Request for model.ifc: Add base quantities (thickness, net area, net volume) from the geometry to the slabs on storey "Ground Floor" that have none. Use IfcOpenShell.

First a look at what the model holds.

```python
import ifcopenshell
import ifcopenshell.util.element
import ifcopenshell.util.unit

model = ifcopenshell.open("model.ifc")
print(model.schema)
for unit_type in ("LENGTHUNIT", "AREAUNIT", "VOLUMEUNIT"):
    print(unit_type, ifcopenshell.util.unit.calculate_unit_scale(model, unit_type))
storey = next(s for s in model.by_type("IfcBuildingStorey") if s.Name == "Ground Floor")
slabs = [e for e in ifcopenshell.util.element.get_decomposition(storey) if e.is_a("IfcSlab")]
for e in sorted(slabs, key=lambda e: e.id()):
    print(e.id(), e.is_a(), e.Name, list(ifcopenshell.util.element.get_psets(e, qtos_only=True)), sep=" | ")
```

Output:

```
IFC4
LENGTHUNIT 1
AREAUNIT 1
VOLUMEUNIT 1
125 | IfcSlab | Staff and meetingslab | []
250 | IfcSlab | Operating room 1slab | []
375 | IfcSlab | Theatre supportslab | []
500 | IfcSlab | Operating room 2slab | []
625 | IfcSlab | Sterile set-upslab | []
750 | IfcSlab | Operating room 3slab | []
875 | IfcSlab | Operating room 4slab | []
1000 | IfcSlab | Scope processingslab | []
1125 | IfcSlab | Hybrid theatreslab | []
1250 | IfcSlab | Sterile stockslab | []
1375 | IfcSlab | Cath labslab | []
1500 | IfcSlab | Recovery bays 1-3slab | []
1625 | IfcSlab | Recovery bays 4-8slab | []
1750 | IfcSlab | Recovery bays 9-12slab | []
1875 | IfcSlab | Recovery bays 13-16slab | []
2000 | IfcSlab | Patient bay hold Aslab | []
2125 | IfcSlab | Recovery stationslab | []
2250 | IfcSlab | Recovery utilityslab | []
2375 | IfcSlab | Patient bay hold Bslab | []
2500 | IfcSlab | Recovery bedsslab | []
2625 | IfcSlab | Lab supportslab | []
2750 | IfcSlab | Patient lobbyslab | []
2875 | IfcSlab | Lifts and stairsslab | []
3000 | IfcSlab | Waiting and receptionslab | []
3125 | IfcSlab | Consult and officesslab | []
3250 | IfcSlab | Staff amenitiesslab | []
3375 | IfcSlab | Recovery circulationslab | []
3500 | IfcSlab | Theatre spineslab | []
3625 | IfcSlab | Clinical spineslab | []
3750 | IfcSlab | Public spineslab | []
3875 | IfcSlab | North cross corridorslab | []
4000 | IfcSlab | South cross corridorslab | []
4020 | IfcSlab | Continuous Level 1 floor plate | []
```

```python
import ifcopenshell
import ifcopenshell.api.pset
import ifcopenshell.geom
import ifcopenshell.util.element
import ifcopenshell.util.shape
import ifcopenshell.util.unit

model = ifcopenshell.open("model.ifc")
unit_scale = ifcopenshell.util.unit.calculate_unit_scale(model)
area_scale = ifcopenshell.util.unit.calculate_unit_scale(model, "AREAUNIT")
volume_scale = ifcopenshell.util.unit.calculate_unit_scale(model, "VOLUMEUNIT")
settings = ifcopenshell.geom.settings()

storey = next(s for s in model.by_type("IfcBuildingStorey") if s.Name == "Ground Floor")
slabs = [e for e in ifcopenshell.util.element.get_decomposition(storey) if e.is_a("IfcSlab")]

for e in sorted(slabs, key=lambda e: e.id()):
    if ifcopenshell.util.element.get_psets(e, qtos_only=True, should_inherit=False):
        continue
    # Geometry comes back in metres, in the element's own axes.
    shape = ifcopenshell.geom.create_shape(settings, e)
    values = {
        "Width": ifcopenshell.util.shape.get_z(shape.geometry) / unit_scale,
        "NetArea": ifcopenshell.util.shape.get_footprint_area(shape.geometry) / area_scale,
        "NetVolume": ifcopenshell.util.shape.get_volume(shape.geometry) / volume_scale,
    }
    qto = ifcopenshell.api.pset.add_qto(model, product=e, name="Qto_SlabBaseQuantities")
    ifcopenshell.api.pset.edit_qto(model, qto=qto, properties=values)
    print(e.id(), {k: round(v, 3) for k, v in values.items()})

model.write("model-out.ifc")
```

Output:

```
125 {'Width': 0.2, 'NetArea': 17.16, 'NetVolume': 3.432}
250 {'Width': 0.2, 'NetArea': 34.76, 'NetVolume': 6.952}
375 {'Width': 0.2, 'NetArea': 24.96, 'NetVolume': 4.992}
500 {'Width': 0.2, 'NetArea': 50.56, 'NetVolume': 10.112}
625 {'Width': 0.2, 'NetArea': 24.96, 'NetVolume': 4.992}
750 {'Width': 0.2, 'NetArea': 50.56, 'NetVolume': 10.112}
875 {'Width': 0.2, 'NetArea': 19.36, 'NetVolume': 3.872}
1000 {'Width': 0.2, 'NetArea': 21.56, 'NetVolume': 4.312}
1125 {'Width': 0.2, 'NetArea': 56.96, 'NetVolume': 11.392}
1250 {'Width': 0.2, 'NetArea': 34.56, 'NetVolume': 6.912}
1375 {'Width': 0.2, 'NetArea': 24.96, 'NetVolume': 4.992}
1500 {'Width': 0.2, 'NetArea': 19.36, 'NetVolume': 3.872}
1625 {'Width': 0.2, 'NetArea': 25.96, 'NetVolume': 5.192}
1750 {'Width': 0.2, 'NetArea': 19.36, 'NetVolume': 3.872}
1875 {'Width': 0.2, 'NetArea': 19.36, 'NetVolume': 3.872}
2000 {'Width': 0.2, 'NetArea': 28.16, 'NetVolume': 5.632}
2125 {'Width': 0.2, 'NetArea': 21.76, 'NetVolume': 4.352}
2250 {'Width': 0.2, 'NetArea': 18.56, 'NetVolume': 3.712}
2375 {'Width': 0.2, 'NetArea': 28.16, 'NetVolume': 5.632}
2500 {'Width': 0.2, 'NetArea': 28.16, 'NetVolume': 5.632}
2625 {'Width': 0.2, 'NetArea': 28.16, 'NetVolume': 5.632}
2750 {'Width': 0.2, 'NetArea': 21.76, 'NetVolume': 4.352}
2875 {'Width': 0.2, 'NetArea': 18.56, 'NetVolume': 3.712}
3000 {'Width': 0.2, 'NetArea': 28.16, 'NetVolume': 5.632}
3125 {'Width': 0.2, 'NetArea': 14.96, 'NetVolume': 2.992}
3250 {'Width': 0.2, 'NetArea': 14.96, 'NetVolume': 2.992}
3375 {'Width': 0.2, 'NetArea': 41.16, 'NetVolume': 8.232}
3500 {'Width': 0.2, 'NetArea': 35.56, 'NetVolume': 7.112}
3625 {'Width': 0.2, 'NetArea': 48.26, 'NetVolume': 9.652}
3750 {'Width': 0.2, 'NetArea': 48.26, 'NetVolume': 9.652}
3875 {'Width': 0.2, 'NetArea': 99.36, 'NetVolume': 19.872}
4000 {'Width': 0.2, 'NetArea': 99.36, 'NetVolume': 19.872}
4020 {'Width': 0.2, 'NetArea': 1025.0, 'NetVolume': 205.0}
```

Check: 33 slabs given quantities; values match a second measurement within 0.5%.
